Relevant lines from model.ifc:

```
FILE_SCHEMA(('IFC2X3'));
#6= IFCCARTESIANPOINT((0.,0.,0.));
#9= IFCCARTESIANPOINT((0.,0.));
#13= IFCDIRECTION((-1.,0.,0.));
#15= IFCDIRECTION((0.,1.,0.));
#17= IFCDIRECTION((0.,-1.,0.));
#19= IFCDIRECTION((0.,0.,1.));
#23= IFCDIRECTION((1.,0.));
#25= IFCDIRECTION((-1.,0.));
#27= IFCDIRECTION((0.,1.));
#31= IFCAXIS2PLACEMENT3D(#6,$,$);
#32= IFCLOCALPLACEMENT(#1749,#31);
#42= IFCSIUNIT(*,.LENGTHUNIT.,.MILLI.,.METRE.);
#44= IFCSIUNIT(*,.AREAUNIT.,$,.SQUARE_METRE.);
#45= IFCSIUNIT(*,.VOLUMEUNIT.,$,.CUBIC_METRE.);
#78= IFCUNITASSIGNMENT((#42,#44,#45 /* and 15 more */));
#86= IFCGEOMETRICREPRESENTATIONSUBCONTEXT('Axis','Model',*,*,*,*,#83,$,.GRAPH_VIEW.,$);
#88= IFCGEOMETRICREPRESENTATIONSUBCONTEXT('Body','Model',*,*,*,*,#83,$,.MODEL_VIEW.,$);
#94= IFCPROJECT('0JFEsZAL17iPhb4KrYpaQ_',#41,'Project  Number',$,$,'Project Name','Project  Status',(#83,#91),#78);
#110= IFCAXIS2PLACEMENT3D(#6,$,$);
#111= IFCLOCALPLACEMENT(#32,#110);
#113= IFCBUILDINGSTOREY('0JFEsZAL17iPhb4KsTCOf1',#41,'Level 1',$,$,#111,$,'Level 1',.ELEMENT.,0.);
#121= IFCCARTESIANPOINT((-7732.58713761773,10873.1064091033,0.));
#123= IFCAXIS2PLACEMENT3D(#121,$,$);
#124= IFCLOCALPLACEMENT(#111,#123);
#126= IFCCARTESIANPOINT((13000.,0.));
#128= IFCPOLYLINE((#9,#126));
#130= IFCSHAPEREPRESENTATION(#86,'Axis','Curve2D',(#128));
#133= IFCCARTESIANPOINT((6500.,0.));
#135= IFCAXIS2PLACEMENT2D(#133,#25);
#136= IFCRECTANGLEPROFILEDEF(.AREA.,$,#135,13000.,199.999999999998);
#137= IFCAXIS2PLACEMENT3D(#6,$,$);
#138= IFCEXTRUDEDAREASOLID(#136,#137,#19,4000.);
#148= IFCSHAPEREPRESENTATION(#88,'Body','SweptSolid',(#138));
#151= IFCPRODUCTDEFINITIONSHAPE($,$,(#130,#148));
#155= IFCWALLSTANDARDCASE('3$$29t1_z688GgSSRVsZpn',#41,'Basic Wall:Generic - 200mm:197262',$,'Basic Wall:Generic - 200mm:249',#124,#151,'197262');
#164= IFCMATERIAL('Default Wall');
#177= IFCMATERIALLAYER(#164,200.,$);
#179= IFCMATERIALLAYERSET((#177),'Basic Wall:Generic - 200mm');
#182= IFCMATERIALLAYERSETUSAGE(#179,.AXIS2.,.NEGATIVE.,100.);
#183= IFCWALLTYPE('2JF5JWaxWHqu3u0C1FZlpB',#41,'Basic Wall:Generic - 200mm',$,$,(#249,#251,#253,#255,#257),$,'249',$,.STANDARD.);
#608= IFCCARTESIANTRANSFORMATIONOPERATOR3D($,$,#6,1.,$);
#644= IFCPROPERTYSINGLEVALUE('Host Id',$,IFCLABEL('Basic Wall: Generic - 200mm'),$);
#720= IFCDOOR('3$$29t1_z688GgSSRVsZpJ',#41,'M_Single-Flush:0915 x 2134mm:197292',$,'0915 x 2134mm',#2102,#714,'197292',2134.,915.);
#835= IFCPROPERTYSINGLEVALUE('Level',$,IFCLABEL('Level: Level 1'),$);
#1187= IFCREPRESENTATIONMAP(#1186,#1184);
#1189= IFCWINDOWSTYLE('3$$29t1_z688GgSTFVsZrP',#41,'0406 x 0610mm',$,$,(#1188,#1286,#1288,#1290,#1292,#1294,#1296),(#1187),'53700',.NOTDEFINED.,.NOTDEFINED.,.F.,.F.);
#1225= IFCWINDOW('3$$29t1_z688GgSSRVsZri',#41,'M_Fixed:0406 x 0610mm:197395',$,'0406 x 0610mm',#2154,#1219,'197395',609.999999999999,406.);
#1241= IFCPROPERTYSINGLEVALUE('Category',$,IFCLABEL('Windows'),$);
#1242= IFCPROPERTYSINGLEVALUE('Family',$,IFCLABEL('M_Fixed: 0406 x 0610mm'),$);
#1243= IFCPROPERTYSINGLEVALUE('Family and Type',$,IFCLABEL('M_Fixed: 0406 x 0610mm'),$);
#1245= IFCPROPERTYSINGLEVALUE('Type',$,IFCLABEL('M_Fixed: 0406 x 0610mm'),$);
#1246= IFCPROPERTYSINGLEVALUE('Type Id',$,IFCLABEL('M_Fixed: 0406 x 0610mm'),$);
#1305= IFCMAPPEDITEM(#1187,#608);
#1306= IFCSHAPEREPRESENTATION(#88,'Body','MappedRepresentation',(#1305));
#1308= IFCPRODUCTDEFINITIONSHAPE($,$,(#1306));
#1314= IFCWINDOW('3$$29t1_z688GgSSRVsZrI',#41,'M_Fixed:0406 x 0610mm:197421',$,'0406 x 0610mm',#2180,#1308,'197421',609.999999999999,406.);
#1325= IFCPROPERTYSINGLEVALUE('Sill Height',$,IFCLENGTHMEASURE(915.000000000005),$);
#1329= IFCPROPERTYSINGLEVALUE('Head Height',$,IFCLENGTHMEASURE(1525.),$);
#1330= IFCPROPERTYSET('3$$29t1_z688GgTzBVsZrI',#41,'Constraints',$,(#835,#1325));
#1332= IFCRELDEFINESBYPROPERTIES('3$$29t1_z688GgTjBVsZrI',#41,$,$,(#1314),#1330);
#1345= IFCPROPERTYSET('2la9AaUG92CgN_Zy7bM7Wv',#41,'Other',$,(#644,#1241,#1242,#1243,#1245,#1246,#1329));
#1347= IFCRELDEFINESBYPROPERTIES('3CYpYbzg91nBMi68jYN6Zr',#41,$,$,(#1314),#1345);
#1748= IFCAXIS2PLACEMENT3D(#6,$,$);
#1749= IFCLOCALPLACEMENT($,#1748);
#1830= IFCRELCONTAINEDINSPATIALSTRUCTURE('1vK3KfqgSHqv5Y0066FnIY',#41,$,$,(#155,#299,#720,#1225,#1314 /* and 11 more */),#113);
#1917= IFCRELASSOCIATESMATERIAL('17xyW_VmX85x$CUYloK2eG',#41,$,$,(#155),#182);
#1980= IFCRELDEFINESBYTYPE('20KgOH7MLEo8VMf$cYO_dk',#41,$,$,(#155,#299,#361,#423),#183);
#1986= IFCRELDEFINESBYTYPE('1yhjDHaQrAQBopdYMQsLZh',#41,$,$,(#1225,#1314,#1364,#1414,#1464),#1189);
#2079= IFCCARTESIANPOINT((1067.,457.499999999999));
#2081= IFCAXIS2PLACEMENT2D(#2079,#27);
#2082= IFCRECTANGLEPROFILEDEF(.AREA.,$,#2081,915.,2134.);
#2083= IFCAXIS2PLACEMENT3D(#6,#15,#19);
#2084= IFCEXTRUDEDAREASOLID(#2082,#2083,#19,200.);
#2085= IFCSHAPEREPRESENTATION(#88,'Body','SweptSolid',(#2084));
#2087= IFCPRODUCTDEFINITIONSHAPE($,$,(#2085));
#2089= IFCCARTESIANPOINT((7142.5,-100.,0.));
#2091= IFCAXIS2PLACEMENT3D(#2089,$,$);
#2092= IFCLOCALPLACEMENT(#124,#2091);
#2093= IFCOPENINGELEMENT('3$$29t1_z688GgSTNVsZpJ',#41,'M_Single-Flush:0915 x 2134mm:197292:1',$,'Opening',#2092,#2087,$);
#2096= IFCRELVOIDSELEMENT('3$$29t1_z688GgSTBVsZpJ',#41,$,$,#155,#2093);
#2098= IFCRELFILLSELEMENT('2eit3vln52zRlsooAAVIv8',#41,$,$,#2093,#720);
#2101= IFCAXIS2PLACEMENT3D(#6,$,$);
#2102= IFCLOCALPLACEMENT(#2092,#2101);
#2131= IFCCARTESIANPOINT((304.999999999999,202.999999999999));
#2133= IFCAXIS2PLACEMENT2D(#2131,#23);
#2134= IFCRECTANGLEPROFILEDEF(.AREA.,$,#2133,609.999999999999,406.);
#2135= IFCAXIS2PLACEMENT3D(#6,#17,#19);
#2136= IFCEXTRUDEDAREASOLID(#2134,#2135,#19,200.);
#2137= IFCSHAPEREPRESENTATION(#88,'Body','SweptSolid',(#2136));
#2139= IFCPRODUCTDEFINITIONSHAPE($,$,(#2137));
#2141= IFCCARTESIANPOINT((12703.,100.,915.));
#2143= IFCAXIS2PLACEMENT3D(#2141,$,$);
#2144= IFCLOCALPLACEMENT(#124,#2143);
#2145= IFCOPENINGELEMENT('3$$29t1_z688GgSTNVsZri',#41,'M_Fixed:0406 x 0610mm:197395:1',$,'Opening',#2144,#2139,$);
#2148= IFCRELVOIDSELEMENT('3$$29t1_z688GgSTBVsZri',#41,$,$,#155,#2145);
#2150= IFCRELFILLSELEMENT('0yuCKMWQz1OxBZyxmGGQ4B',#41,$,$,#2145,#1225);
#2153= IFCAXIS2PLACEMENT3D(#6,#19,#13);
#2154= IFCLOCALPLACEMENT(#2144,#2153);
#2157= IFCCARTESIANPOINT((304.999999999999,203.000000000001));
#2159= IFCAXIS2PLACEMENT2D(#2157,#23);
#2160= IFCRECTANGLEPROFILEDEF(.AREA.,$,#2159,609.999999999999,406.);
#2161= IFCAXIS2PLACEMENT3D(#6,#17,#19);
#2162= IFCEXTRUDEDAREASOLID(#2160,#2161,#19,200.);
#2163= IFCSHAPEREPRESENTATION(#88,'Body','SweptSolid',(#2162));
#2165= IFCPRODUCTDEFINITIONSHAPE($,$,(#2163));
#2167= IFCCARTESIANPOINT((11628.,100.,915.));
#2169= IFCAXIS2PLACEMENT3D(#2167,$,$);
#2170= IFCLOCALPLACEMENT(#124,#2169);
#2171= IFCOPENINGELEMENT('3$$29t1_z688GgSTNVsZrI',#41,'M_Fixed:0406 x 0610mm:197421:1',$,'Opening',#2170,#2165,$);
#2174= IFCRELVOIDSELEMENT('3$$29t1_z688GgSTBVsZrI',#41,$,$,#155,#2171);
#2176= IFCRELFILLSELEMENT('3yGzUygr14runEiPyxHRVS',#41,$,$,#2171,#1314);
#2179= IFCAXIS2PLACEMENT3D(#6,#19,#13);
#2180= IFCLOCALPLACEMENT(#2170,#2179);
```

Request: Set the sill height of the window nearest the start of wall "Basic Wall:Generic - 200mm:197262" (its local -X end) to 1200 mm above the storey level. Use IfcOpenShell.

```python
import numpy as np
import ifcopenshell
import ifcopenshell.api.geometry
import ifcopenshell.api.pset
import ifcopenshell.geom
import ifcopenshell.util.element
import ifcopenshell.util.placement
import ifcopenshell.util.shape
import ifcopenshell.util.unit

model = ifcopenshell.open("model.ifc")
unit_scale = ifcopenshell.util.unit.calculate_unit_scale(model)

window = model.by_guid("3$$29t1_z688GgSSRVsZrI")
opening = window.FillsVoids[0].RelatingOpeningElement
storey = ifcopenshell.util.element.get_container(window, ifc_class="IfcBuildingStorey")
level = ifcopenshell.util.placement.get_local_placement(storey.ObjectPlacement)[2, 3]

# The opening's origin need not be at the sill, so measure its lowest point.
shape = ifcopenshell.geom.create_shape(ifcopenshell.geom.settings(), opening)
bottom = ifcopenshell.util.shape.get_shape_bottom_elevation(shape, shape.geometry) / unit_scale
dz = level + 1200.0 - bottom

shift = np.array([0.0, 0.0, dz])
# The window is placed relative to its opening, so it follows when the opening moves.
matrix = ifcopenshell.util.placement.get_local_placement(opening.ObjectPlacement)
matrix[:3, 3] += shift
ifcopenshell.api.geometry.edit_object_placement(
    model, product=opening, matrix=matrix, is_si=False, should_transform_children=True
)

# Keep the stored heights in step.
pset = model.by_id(ifcopenshell.util.element.get_pset(window, "Constraints", should_inherit=False)["id"])
ifcopenshell.api.pset.edit_pset(model, pset=pset, properties={
    "Sill Height": model.create_entity("IfcLengthMeasure", ifcopenshell.util.element.get_pset(window, "Constraints", "Sill Height") + dz),
})
pset = model.by_id(ifcopenshell.util.element.get_pset(window, "Other", should_inherit=False)["id"])
ifcopenshell.api.pset.edit_pset(model, pset=pset, properties={
    "Head Height": model.create_entity("IfcLengthMeasure", ifcopenshell.util.element.get_pset(window, "Other", "Head Height") + dz),
})

print(f"moved by {dz * unit_scale:+.3f} m")

model.write("model_v2.ifc")
```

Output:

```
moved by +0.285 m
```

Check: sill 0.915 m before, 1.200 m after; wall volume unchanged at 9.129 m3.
